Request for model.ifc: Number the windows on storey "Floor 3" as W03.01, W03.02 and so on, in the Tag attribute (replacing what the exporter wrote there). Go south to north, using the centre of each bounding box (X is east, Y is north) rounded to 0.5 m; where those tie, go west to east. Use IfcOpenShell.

First a look at what the model holds.

```python
import ifcopenshell
import ifcopenshell.util.element
import ifcopenshell.util.placement

model = ifcopenshell.open("model.ifc")
print(model.schema)
storey = next(s for s in model.by_type("IfcBuildingStorey") if s.Name == "Floor 3")
windows = [e for e in ifcopenshell.util.element.get_decomposition(storey) if e.is_a("IfcWindow")]
for e in sorted(windows, key=lambda e: e.id()):
    origin = ifcopenshell.util.placement.get_local_placement(e.ObjectPlacement)[:3, 3]
    print(e.id(), e.Tag, e.Name, origin.round(2) + 0.0, sep=" | ")
```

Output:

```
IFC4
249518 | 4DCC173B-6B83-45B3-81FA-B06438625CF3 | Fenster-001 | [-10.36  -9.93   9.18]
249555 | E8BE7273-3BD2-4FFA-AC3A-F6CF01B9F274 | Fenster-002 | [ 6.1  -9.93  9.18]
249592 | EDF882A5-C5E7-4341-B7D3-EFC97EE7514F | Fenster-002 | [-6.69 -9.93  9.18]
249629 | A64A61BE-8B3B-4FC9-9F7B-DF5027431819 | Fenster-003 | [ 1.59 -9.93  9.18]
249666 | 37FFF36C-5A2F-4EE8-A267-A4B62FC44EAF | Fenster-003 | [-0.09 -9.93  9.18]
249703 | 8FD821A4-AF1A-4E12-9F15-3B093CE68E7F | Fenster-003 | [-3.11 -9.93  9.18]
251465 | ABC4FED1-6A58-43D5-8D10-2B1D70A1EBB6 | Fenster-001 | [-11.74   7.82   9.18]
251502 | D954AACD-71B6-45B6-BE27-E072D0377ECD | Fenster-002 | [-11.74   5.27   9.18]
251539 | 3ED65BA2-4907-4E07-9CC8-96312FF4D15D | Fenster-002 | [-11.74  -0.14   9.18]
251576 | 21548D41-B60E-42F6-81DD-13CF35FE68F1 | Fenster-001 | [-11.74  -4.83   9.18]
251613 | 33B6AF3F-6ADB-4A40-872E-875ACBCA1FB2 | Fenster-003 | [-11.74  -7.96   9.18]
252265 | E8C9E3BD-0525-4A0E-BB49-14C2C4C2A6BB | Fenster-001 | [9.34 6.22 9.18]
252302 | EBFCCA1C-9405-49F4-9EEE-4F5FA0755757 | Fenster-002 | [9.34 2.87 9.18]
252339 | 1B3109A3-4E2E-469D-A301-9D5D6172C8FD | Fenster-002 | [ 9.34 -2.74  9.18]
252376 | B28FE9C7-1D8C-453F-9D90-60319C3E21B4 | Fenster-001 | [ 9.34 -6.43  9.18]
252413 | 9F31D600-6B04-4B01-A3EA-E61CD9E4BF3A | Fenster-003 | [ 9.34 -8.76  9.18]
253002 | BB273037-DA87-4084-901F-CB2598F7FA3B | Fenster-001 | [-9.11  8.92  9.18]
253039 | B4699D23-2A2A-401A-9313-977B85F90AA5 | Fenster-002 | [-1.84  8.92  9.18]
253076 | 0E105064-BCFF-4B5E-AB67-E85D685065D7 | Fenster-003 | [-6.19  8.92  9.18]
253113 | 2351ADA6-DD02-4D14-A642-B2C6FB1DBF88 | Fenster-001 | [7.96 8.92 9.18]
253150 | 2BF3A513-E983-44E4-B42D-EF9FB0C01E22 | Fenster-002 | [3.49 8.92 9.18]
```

```python
import ifcopenshell
import ifcopenshell.geom
import ifcopenshell.util.element
import ifcopenshell.util.shape

model = ifcopenshell.open("model.ifc")
settings = ifcopenshell.geom.settings()
settings.set("use-world-coords", True)


def centre(element):
    shape = ifcopenshell.geom.create_shape(settings, element)
    return ifcopenshell.util.shape.get_bbox_centroid(shape.geometry)


storey = next(s for s in model.by_type("IfcBuildingStorey") if s.Name == "Floor 3")
windows = [e for e in ifcopenshell.util.element.get_decomposition(storey) if e.is_a("IfcWindow")]

# Insertion points can sit at a corner or the storey origin, so sort by the geometry (in metres).
centres = {e: centre(e) for e in windows}
windows.sort(key=lambda e: (round(centres[e][1] / 0.5), centres[e][0]))

for i, e in enumerate(windows, start=1):
    number = f"W03.{i:02d}"
    e.Tag = number
    print(e.id(), number)

model.write("model_updated.ifc")
```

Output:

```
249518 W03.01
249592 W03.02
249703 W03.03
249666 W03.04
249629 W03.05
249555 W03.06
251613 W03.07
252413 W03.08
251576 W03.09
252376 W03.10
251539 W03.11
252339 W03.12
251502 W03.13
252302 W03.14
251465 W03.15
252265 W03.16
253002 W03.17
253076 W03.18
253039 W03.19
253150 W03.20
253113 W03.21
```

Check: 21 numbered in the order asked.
